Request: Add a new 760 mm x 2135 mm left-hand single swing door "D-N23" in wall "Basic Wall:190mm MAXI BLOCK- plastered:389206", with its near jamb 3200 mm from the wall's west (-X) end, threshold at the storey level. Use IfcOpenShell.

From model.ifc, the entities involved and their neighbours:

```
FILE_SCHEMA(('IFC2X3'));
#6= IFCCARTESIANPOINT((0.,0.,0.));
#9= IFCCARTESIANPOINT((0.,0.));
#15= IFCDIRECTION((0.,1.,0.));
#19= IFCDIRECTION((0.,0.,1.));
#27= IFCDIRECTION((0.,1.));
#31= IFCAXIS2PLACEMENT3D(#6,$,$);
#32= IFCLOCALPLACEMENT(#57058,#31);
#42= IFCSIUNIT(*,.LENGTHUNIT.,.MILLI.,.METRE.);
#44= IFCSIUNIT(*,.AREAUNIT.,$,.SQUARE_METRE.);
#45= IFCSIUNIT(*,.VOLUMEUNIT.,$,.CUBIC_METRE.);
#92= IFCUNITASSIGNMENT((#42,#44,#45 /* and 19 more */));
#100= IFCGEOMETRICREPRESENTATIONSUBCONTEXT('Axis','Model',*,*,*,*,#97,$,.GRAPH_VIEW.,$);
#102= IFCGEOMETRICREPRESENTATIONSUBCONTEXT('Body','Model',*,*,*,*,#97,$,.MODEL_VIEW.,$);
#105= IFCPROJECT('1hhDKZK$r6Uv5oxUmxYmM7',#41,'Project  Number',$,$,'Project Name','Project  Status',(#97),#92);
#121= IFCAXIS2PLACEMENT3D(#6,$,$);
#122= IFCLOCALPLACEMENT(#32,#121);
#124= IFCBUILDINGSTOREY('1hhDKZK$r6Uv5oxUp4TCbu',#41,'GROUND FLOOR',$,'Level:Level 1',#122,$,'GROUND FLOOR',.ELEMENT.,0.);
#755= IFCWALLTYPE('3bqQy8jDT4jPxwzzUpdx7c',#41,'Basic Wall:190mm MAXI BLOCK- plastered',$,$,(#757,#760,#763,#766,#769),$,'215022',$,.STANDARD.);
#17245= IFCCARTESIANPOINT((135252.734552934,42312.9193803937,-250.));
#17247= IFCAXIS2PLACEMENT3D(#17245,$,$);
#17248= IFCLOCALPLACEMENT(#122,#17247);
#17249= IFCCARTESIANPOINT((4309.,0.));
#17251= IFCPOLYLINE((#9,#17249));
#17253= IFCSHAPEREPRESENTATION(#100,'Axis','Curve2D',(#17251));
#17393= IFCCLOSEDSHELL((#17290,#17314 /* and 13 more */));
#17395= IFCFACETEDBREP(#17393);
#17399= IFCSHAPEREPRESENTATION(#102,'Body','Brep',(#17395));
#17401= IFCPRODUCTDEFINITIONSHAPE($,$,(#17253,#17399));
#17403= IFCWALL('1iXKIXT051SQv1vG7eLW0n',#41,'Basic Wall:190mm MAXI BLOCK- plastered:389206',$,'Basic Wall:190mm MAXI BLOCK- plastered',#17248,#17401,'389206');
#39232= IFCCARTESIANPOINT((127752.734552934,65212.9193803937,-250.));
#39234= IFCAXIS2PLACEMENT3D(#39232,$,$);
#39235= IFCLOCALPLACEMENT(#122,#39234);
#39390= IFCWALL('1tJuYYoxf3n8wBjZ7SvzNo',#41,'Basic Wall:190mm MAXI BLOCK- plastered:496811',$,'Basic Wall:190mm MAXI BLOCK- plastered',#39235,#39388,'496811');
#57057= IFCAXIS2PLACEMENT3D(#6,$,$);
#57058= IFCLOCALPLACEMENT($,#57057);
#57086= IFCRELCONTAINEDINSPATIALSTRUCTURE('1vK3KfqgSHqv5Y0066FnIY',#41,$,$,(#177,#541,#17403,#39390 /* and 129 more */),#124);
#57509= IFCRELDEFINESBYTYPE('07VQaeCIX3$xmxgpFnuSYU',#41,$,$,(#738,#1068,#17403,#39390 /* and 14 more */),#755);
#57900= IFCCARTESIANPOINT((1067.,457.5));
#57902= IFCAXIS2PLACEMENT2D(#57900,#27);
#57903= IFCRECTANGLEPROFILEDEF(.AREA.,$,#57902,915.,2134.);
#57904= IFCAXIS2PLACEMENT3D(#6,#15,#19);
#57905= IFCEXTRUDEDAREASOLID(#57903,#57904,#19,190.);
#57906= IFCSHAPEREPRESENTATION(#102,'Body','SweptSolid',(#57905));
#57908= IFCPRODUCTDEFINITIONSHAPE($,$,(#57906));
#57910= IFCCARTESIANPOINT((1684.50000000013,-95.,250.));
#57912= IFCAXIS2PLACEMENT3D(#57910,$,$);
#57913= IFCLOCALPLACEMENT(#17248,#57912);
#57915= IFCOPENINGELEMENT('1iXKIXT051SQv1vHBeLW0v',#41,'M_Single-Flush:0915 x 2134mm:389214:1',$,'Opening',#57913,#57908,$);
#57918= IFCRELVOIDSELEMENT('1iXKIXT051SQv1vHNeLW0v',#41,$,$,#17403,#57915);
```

```python
import numpy as np
import ifcopenshell
import ifcopenshell.api.feature
import ifcopenshell.api.geometry
import ifcopenshell.api.root
import ifcopenshell.api.spatial
import ifcopenshell.api.type
import ifcopenshell.geom
import ifcopenshell.util.element
import ifcopenshell.util.placement
import ifcopenshell.util.representation
import ifcopenshell.util.shape
import ifcopenshell.util.unit

model = ifcopenshell.open("model.ifc")
unit_scale = ifcopenshell.util.unit.calculate_unit_scale(model)
settings = ifcopenshell.geom.settings()


def volume(element):
    """Net volume in cubic metres, openings subtracted."""
    shape = ifcopenshell.geom.create_shape(settings, element)
    return ifcopenshell.util.shape.get_volume(shape.geometry)


wall = model.by_id(17403)
storey = ifcopenshell.util.element.get_container(wall, ifc_class="IfcBuildingStorey")
context = ifcopenshell.util.representation.get_context(model, "Model", "Body", "MODEL_VIEW")
before = volume(wall)

width, height, from_end, sill = 0.76, 2.135, 3.2, 0.0  # metres

# The wall runs along its own X axis, and the end named is its -X end.
wall_shape = ifcopenshell.geom.create_shape(settings, wall)
x, y, z = ifcopenshell.util.shape.get_vertices(wall_shape.geometry).T
start = x.min() + from_end
face, thickness = float(y.min()), float(y.max() - y.min())
wall_matrix = ifcopenshell.util.placement.get_local_placement(wall.ObjectPlacement)
level = ifcopenshell.util.placement.get_local_placement(storey.ObjectPlacement)[2, 3]


def in_wall(x, y):
    """Placement at x, y metres in the wall's axes, at sill height."""
    matrix = wall_matrix.copy()
    matrix[:, 3] = wall_matrix @ np.array([x / unit_scale, y / unit_scale, 0.0, 1.0])
    matrix[2, 3] = level + sill / unit_scale
    return matrix


# Opening: a box that overshoots both wall faces by 50 mm.
opening = ifcopenshell.api.root.create_entity(model, ifc_class="IfcOpeningElement")
box = ifcopenshell.api.geometry.add_wall_representation(
    model, context=context, length=width, height=height, thickness=thickness + 0.1
)
ifcopenshell.api.geometry.assign_representation(model, product=opening, representation=box)
ifcopenshell.api.geometry.edit_object_placement(model, product=opening, matrix=in_wall(start, face - 0.05), is_si=False)
ifcopenshell.api.feature.add_feature(model, feature=opening, element=wall)

door = ifcopenshell.api.root.create_entity(model, ifc_class="IfcDoor", name="D-N23")
door.OverallWidth, door.OverallHeight = width / unit_scale, height / unit_scale
body = ifcopenshell.api.geometry.add_door_representation(
    model,
    context=context,
    overall_width=door.OverallWidth,
    overall_height=door.OverallHeight,
    operation_type="SINGLE_SWING_LEFT",
    lining_properties={"LiningDepth": thickness / unit_scale, "ThresholdDepth": thickness / unit_scale},
)
ifcopenshell.api.geometry.assign_representation(model, product=door, representation=body)
ifcopenshell.api.spatial.assign_container(model, products=[door], relating_structure=storey)
fills = ifcopenshell.api.feature.add_filling(model, opening=opening, element=door)
fills.OwnerHistory = door.OwnerHistory  # required in IFC2X3

# IFC2X3 keeps the operation on the door style.
style = ifcopenshell.api.root.create_entity(model, ifc_class="IfcDoorStyle", name="D-N23")
style.OperationType, style.ConstructionType = "SINGLE_SWING_LEFT", "NOTDEFINED"
style.ParameterTakesPrecedence = style.Sizeable = False
ifcopenshell.api.type.assign_type(model, related_objects=[door], relating_type=style)

# The lining spans the wall, so the door starts at the wall face.
ifcopenshell.api.geometry.edit_object_placement(model, product=door, matrix=in_wall(start, face), is_si=False)

after = volume(wall)

print(f"wall volume {before:.3f} -> {after:.3f} m3")

model.write("model_edited.ifc")
```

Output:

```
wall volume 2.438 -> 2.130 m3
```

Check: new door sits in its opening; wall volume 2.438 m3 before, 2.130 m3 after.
